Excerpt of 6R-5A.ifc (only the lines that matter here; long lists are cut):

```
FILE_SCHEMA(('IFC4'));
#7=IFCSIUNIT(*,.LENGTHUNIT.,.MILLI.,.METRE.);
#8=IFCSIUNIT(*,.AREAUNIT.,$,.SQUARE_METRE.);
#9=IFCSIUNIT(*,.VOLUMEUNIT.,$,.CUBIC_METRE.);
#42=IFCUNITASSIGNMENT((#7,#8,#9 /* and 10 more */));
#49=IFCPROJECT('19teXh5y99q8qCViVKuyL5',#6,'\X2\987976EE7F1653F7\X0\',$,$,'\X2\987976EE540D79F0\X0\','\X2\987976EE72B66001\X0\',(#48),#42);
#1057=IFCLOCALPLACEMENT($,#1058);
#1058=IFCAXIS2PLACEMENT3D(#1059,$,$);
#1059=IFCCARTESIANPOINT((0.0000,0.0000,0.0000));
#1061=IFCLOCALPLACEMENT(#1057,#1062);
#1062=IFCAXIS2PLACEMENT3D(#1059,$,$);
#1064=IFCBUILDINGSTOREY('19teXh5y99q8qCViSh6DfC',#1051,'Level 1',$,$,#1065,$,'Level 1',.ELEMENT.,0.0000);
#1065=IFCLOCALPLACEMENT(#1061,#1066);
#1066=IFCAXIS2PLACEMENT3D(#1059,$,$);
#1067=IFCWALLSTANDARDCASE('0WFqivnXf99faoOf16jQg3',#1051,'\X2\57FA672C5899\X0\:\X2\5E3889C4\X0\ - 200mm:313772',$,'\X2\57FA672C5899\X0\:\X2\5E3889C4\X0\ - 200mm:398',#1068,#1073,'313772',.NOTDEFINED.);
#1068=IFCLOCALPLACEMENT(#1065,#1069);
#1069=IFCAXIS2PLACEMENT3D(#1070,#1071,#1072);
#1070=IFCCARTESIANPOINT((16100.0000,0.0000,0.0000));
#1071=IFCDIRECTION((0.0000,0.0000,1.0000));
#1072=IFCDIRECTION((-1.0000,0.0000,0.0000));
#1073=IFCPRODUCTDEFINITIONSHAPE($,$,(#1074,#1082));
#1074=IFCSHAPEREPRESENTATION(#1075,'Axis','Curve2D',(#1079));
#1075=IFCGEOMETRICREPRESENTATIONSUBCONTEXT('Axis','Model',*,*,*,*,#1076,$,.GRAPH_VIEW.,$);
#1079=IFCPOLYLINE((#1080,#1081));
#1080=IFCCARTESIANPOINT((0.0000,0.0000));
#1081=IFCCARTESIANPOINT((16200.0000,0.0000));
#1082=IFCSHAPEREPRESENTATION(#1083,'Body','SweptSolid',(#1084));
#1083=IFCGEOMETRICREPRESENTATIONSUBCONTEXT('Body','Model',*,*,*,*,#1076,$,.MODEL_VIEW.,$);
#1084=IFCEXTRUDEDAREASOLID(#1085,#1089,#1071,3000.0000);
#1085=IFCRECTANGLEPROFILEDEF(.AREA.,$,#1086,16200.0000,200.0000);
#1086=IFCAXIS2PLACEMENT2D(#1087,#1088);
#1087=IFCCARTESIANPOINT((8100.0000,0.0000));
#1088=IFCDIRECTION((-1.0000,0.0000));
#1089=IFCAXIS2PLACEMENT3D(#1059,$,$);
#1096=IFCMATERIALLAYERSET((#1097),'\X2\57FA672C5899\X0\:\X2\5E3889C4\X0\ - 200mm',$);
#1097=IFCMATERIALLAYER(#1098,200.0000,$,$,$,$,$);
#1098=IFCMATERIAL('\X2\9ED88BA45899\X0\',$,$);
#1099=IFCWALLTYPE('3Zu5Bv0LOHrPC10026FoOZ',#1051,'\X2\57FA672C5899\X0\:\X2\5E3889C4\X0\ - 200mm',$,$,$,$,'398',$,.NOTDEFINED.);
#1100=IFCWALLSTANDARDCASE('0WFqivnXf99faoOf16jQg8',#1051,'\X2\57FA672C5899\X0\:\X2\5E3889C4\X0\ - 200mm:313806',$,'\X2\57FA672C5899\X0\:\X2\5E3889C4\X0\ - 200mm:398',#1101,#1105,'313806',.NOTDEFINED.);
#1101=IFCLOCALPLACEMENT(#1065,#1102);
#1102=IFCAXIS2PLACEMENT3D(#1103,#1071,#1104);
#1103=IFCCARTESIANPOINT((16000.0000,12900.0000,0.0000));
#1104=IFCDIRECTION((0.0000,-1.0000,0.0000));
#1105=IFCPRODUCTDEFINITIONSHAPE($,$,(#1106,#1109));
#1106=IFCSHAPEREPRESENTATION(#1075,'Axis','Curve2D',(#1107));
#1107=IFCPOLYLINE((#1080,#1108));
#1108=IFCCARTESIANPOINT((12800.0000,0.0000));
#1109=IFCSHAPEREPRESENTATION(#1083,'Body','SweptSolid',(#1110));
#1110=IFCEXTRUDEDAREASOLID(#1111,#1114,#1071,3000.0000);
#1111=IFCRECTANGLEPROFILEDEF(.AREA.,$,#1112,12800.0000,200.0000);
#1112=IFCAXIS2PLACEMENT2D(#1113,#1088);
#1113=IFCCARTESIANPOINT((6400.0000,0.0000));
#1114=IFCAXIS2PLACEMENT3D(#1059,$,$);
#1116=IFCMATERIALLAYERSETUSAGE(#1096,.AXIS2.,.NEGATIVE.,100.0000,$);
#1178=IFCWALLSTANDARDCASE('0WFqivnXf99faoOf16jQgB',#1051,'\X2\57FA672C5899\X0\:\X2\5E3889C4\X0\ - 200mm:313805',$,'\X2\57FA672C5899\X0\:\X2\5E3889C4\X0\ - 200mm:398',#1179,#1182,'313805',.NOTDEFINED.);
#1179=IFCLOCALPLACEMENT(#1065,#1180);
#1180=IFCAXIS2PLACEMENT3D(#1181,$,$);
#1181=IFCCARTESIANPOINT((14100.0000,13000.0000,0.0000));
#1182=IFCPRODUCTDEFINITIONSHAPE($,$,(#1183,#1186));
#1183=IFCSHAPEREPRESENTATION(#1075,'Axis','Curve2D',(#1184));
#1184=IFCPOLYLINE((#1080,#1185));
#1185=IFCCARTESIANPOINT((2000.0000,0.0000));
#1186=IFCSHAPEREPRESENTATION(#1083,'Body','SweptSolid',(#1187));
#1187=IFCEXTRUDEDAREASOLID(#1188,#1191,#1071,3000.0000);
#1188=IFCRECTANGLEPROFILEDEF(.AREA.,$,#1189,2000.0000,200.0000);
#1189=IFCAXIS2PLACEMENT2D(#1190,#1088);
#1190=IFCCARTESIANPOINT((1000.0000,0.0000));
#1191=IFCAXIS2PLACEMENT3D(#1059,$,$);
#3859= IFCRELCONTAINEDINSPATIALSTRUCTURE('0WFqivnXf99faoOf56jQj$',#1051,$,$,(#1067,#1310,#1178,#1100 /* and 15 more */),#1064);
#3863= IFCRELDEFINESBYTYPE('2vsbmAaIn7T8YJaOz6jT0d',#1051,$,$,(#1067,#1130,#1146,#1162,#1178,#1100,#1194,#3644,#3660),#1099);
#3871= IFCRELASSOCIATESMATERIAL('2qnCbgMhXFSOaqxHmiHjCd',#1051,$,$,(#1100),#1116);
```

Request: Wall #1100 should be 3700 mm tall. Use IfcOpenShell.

```python
import ifcopenshell
import ifcopenshell.geom
import ifcopenshell.util.representation
import ifcopenshell.util.shape

model = ifcopenshell.open("6R-5A.ifc")
settings = ifcopenshell.geom.settings()


def volume(element):
    """Net volume in cubic metres, openings subtracted."""
    shape = ifcopenshell.geom.create_shape(settings, element)
    return ifcopenshell.util.shape.get_volume(shape.geometry)


wall = model.by_id(1100)
before = volume(wall)

body = ifcopenshell.util.representation.get_representation(wall, "Model", "Body")
solid = body.Items[0]
old_height = solid.Depth
solid.Depth = 3700.0
after = volume(wall)

print(f"height {old_height:g} -> {solid.Depth:g}, volume {before:.3f} -> {after:.3f} m3")

model.write("6R-5A_updated.ifc")
```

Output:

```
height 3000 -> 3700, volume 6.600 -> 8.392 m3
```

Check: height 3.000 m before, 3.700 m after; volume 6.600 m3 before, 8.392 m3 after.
